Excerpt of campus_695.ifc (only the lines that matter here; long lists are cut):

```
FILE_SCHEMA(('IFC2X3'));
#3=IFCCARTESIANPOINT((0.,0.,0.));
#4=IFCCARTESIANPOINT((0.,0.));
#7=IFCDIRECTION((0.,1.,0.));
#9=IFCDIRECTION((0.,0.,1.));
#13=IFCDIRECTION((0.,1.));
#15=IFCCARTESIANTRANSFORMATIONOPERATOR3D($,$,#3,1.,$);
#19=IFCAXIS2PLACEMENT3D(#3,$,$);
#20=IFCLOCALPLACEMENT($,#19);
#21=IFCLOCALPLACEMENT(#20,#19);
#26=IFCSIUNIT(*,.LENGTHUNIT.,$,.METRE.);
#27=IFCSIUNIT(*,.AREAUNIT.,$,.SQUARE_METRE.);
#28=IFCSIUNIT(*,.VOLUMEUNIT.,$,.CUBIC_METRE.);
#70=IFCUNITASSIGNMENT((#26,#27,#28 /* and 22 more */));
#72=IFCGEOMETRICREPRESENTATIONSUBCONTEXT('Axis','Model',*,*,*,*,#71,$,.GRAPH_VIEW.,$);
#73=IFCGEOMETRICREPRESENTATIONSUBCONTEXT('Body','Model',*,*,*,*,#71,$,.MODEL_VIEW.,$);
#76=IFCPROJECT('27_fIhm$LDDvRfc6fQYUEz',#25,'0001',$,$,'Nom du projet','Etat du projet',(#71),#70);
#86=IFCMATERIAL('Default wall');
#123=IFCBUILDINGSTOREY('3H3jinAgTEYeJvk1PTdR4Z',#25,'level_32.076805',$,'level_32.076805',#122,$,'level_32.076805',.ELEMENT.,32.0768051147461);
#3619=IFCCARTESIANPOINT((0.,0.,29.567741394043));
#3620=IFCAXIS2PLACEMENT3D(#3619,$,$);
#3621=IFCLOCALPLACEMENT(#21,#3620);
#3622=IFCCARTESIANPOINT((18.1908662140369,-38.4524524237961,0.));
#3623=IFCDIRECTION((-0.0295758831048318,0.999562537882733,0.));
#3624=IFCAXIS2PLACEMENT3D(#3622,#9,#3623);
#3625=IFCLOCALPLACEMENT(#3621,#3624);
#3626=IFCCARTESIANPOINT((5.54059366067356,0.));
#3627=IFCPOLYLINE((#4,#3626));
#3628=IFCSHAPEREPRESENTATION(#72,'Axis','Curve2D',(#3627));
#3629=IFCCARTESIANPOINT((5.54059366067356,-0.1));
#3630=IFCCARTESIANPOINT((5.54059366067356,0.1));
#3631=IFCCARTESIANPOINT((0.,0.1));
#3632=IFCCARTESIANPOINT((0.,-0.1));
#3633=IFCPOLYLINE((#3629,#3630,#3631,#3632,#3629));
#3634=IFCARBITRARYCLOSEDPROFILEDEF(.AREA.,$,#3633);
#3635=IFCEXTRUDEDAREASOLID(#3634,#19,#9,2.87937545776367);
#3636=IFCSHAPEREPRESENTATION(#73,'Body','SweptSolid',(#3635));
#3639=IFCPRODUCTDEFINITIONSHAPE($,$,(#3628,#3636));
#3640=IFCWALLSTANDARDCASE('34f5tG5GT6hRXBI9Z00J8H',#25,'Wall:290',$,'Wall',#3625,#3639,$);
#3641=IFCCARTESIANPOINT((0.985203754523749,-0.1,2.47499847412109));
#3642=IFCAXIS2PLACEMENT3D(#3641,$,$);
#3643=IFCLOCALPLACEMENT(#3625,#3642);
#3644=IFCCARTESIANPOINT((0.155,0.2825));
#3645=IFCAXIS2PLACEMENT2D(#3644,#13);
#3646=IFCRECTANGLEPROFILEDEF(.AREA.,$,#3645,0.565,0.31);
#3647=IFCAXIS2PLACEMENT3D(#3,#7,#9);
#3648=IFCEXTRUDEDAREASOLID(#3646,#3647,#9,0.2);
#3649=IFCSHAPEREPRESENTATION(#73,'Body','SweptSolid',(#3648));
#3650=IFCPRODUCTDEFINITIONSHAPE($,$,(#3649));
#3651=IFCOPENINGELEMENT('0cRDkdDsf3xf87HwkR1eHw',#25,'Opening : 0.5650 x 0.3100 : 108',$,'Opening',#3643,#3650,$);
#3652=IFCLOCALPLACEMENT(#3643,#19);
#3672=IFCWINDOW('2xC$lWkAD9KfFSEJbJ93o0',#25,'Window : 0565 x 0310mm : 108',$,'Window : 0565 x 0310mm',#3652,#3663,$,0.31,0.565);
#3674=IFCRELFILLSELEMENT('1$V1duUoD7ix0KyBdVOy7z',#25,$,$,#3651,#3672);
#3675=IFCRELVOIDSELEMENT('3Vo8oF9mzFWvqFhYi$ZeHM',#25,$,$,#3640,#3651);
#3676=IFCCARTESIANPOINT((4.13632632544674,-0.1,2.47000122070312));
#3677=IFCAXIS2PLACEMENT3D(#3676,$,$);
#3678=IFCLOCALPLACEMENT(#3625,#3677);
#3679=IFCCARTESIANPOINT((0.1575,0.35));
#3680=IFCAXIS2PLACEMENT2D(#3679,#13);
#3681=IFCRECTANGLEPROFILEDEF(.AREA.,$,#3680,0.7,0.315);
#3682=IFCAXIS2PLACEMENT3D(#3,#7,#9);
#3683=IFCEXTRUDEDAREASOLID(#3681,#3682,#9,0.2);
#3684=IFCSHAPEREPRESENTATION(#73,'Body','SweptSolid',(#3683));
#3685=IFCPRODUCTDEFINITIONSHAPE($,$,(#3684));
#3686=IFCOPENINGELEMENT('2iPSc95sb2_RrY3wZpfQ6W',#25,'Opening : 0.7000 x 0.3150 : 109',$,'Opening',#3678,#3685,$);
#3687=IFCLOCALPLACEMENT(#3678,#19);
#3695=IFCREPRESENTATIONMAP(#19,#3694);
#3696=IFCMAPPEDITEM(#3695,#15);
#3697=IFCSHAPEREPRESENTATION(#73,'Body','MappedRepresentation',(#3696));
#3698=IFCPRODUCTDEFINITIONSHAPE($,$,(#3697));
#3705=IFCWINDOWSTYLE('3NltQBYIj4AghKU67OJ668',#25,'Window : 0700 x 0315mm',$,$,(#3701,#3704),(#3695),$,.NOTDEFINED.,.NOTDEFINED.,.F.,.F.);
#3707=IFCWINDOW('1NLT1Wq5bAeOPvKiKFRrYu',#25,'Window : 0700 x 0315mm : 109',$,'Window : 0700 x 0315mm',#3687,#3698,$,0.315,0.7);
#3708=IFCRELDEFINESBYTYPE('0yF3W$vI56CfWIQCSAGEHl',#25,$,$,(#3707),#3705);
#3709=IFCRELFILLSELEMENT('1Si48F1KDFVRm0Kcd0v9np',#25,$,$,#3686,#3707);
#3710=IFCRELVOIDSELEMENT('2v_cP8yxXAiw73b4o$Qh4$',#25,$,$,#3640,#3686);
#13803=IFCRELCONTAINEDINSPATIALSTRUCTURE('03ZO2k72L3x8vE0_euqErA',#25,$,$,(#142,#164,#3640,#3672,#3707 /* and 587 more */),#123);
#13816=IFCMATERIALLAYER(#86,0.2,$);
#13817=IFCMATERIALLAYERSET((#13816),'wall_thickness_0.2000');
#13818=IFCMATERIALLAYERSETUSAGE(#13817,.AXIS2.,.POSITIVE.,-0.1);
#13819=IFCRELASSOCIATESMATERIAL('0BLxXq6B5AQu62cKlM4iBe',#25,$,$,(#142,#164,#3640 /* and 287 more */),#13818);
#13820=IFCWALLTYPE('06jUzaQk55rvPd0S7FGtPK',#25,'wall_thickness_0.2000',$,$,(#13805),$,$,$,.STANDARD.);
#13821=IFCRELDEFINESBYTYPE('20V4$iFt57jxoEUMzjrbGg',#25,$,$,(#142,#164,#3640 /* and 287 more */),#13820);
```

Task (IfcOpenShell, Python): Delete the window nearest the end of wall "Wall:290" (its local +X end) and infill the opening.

```python
import ifcopenshell
import ifcopenshell.api.feature
import ifcopenshell.api.root
import ifcopenshell.geom
import ifcopenshell.util.shape

model = ifcopenshell.open("campus_695.ifc")
settings = ifcopenshell.geom.settings()


def volume(element):
    """Net volume in cubic metres, openings subtracted."""
    shape = ifcopenshell.geom.create_shape(settings, element)
    return ifcopenshell.util.shape.get_volume(shape.geometry)


window = model.by_guid("1NLT1Wq5bAeOPvKiKFRrYu")
opening = window.FillsVoids[0].RelatingOpeningElement
wall = opening.VoidsElements[0].RelatingBuildingElement
before = volume(wall)

ifcopenshell.api.root.remove_product(model, product=window)
ifcopenshell.api.feature.remove_feature(model, feature=opening)

after = volume(wall)

print(f"wall volume {before:.3f} -> {after:.3f} m3")

model.write("campus_695_rev.ifc")
```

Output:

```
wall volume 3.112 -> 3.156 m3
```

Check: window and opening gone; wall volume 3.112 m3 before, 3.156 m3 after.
